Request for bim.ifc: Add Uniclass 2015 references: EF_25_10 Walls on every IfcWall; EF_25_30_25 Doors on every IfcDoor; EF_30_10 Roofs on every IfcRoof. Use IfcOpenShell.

First a look at what the model holds.

```python
import ifcopenshell

model = ifcopenshell.open("bim.ifc")
print(model.schema)
print("classifications:", [c.Name for c in model.by_type("IfcClassification")])
for ifc_class in ("IfcDoor", "IfcRoof", "IfcStair", "IfcWall", "IfcWindow"):
    print(ifc_class, len(model.by_type(ifc_class)))
```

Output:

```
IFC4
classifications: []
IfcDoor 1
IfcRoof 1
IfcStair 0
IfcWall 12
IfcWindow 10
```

```python
import ifcopenshell
import ifcopenshell.api.classification

model = ifcopenshell.open("bim.ifc")

system = ifcopenshell.api.classification.add_classification(model, classification="Uniclass 2015")

codes = {
    "IfcWall": ("EF_25_10", "Walls"),
    "IfcDoor": ("EF_25_30_25", "Doors"),
    "IfcRoof": ("EF_30_10", "Roofs"),
}
for ifc_class, (code, name) in codes.items():
    products = model.by_type(ifc_class)
    ifcopenshell.api.classification.add_reference(
        model, products=products, classification=system, identification=code, name=name
    )
    print(code, len(products))

model.write("bim_v2.ifc")
```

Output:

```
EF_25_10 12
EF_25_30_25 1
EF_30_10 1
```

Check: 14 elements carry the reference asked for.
